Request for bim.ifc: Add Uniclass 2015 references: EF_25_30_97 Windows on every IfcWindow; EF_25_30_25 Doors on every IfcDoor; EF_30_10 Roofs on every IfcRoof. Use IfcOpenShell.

First a look at what the model holds.

```python
import ifcopenshell

model = ifcopenshell.open("bim.ifc")
print(model.schema)
print("classifications:", [c.Name for c in model.by_type("IfcClassification")])
for ifc_class in ("IfcDoor", "IfcRoof", "IfcStair", "IfcWall", "IfcWindow"):
    print(ifc_class, len(model.by_type(ifc_class)))
```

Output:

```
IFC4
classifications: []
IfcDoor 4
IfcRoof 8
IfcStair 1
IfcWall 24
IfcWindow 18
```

```python
import ifcopenshell
import ifcopenshell.api.classification

model = ifcopenshell.open("bim.ifc")

system = ifcopenshell.api.classification.add_classification(model, classification="Uniclass 2015")

codes = {
    "IfcWindow": ("EF_25_30_97", "Windows"),
    "IfcDoor": ("EF_25_30_25", "Doors"),
    "IfcRoof": ("EF_30_10", "Roofs"),
}
for ifc_class, (code, name) in codes.items():
    products = model.by_type(ifc_class)
    ifcopenshell.api.classification.add_reference(
        model, products=products, classification=system, identification=code, name=name
    )
    print(code, len(products))

model.write("bim-out.ifc")
```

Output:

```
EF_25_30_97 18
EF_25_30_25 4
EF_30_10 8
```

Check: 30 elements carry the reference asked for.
